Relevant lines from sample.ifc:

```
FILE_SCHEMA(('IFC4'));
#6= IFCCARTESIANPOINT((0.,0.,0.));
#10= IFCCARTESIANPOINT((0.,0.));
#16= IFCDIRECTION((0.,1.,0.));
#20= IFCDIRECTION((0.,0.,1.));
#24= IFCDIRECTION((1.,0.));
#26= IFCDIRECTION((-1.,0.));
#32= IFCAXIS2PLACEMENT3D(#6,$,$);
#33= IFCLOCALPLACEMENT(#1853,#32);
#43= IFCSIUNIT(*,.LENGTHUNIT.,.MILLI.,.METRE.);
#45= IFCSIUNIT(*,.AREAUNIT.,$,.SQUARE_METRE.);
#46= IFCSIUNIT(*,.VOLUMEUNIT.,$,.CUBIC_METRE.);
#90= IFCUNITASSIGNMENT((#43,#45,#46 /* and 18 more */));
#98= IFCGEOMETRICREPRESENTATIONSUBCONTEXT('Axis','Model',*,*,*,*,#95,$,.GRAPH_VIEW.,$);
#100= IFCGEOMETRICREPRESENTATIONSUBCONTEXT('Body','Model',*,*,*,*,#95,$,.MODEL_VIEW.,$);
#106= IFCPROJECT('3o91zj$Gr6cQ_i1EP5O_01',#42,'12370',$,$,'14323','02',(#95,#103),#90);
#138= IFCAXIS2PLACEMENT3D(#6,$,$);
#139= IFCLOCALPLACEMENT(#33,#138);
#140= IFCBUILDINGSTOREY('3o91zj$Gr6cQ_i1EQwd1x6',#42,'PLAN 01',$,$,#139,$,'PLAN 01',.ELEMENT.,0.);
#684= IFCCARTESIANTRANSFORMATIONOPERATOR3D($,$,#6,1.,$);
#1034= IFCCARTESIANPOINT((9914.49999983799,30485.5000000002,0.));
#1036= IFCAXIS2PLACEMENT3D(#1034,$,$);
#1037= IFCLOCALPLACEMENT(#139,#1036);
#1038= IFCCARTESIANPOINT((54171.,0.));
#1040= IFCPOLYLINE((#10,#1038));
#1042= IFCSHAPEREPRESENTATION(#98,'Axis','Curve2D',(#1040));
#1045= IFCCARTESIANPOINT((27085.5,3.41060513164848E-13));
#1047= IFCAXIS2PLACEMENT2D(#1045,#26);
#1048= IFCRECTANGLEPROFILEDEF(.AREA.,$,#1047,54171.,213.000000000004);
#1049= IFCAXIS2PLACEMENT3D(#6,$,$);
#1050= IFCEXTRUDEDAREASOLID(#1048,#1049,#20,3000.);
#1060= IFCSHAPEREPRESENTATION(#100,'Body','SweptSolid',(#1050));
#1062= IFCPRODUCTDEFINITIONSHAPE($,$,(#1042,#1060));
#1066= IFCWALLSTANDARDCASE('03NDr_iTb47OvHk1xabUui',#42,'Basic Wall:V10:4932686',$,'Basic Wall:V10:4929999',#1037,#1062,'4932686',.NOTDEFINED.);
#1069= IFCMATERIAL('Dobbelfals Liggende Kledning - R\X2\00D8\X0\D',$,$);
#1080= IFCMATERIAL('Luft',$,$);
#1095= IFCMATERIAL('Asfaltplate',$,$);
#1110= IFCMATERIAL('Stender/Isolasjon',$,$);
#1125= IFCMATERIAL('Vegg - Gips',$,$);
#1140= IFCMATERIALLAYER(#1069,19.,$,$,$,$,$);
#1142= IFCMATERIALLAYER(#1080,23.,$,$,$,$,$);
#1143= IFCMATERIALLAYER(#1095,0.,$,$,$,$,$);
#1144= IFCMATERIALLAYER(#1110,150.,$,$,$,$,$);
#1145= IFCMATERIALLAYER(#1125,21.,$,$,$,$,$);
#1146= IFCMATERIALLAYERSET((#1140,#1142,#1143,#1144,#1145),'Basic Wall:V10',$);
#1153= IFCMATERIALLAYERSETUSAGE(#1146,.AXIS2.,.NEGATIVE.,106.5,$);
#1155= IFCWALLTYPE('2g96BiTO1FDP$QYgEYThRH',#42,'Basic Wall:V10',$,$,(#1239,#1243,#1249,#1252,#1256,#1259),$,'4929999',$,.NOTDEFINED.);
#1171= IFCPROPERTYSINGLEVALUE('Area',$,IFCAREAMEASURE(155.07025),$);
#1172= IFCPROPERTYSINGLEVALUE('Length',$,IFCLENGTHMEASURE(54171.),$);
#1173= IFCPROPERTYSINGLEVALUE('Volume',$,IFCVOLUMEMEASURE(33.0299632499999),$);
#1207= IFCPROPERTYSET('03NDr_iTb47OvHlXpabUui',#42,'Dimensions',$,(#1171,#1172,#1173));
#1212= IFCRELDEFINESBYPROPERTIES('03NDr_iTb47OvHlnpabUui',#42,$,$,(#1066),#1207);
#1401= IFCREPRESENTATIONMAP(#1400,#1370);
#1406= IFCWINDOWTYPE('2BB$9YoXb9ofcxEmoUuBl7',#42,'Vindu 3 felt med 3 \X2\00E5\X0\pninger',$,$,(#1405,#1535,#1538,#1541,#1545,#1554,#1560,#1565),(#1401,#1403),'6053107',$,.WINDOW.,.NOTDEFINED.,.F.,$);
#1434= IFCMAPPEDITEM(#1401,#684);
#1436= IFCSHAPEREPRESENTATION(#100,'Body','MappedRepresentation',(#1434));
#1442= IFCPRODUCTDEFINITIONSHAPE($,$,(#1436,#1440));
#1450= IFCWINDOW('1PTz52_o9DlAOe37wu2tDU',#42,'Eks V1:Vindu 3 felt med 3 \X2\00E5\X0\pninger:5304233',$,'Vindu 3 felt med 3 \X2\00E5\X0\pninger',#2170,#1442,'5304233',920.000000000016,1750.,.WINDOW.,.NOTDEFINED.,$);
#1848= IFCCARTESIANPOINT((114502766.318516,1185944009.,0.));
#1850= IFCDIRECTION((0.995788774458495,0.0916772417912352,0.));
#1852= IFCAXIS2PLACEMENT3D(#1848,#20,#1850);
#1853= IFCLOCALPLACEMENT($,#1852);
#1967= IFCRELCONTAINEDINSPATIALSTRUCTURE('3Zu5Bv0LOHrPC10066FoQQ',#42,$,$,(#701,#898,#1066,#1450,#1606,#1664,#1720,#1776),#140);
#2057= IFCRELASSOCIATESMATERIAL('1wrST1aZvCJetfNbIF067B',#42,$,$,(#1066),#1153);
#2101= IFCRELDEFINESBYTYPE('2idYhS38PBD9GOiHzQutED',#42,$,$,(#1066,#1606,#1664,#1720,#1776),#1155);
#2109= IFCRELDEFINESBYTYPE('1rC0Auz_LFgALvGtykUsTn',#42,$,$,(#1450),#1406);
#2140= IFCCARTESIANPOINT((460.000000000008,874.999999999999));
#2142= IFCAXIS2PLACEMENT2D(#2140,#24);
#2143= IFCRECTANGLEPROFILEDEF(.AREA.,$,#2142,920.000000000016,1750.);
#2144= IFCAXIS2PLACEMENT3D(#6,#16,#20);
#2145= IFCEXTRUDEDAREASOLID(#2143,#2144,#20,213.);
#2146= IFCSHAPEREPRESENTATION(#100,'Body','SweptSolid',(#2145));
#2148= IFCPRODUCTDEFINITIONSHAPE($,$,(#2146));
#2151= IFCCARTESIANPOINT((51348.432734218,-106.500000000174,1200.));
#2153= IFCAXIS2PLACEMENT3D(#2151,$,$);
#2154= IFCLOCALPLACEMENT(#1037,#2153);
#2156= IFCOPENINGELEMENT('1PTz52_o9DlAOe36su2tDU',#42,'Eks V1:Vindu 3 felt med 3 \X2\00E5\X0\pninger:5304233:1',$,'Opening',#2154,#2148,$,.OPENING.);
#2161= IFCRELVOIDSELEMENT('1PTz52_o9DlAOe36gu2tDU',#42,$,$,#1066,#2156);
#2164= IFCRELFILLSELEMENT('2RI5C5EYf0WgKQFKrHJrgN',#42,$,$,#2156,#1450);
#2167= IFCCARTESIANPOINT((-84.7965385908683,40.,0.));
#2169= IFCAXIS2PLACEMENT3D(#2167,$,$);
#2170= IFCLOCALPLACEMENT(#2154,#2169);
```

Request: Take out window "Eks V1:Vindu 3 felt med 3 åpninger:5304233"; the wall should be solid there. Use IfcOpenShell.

```python
import ifcopenshell
import ifcopenshell.api.feature
import ifcopenshell.api.pset
import ifcopenshell.api.root
import ifcopenshell.geom
import ifcopenshell.util.element
import ifcopenshell.util.shape
import ifcopenshell.util.unit

model = ifcopenshell.open("sample.ifc")
area_scale = ifcopenshell.util.unit.calculate_unit_scale(model, "AREAUNIT")
volume_scale = ifcopenshell.util.unit.calculate_unit_scale(model, "VOLUMEUNIT")
settings = ifcopenshell.geom.settings()


def volume(element):
    """Net volume in cubic metres, openings subtracted."""
    shape = ifcopenshell.geom.create_shape(settings, element)
    return ifcopenshell.util.shape.get_volume(shape.geometry)


window = model.by_guid("1PTz52_o9DlAOe37wu2tDU")
opening = window.FillsVoids[0].RelatingOpeningElement
wall = opening.VoidsElements[0].RelatingBuildingElement
before = volume(wall)

ifcopenshell.api.root.remove_product(model, product=window)
ifcopenshell.api.feature.remove_feature(model, feature=opening)

after = volume(wall)
thickness = 0.213  # wall thickness in metres

# Update the wall's stored quantities.
pset = model.by_id(ifcopenshell.util.element.get_pset(wall, "Dimensions", should_inherit=False)["id"])
ifcopenshell.api.pset.edit_pset(model, pset=pset, properties={
    "Area": model.create_entity("IfcAreaMeasure", after / thickness / area_scale),
    "Volume": model.create_entity("IfcVolumeMeasure", after / volume_scale),
})

print(f"wall volume {before:.3f} -> {after:.3f} m3")

model.write("sample_edited.ifc")
```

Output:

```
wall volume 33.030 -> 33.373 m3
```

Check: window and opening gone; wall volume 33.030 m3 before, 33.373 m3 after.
